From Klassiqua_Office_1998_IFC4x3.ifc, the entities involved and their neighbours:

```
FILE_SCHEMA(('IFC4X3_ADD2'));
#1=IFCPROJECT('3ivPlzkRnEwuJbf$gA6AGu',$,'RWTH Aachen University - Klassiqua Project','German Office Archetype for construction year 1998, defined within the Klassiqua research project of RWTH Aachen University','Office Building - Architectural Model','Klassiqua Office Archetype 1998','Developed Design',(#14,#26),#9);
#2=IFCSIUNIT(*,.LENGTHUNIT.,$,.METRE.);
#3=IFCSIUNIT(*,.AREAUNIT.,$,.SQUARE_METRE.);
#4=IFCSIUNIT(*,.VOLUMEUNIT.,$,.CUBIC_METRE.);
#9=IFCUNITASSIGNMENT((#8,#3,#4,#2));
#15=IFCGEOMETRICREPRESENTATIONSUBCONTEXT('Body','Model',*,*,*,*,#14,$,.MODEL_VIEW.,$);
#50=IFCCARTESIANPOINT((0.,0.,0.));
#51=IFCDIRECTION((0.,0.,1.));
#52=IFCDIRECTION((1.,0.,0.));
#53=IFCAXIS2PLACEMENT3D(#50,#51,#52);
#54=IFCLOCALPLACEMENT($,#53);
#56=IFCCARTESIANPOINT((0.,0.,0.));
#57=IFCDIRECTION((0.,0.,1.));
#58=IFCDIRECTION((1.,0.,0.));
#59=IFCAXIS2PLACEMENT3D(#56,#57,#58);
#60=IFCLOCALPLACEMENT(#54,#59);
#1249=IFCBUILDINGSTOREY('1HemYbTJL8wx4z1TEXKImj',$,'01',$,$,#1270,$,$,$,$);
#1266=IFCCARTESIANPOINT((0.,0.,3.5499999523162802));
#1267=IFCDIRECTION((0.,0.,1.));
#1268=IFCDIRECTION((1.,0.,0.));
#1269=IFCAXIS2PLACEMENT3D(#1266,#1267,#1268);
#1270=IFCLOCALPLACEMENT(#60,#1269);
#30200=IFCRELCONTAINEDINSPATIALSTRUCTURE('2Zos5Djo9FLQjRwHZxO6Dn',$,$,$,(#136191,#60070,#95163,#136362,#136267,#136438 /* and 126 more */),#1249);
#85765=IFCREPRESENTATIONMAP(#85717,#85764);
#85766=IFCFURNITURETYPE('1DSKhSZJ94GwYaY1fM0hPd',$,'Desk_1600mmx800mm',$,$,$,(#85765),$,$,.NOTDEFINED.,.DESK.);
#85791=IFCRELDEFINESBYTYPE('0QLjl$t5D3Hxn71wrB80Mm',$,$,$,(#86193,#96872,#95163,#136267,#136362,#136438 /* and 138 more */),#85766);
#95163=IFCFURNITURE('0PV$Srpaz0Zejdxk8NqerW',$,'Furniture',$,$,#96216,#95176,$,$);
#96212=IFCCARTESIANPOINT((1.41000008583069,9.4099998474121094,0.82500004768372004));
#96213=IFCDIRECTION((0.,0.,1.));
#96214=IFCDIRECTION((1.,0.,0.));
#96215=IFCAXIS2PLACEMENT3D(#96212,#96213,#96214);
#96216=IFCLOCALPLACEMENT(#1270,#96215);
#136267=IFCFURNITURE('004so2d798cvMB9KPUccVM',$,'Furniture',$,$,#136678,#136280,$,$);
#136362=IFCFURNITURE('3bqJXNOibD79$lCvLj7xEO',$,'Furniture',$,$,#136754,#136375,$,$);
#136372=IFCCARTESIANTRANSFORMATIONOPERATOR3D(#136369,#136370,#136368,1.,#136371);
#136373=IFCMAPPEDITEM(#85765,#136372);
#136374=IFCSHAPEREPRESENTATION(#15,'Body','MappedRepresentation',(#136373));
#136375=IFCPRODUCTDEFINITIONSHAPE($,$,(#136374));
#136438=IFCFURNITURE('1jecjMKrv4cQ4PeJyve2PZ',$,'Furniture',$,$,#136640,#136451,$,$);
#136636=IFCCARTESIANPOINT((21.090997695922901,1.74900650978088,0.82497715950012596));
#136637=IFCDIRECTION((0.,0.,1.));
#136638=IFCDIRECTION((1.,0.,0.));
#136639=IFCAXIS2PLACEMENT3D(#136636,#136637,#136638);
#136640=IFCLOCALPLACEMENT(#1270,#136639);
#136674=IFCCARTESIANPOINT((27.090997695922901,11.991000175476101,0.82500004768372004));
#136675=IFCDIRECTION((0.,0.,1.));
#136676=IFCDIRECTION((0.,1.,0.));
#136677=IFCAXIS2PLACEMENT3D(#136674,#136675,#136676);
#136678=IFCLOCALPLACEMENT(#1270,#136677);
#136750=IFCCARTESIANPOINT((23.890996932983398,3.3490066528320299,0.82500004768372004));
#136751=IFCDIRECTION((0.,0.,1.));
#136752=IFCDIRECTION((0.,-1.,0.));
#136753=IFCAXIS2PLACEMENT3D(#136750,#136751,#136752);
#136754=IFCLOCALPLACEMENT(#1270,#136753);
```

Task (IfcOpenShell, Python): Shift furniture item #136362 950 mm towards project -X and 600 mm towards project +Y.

```python
import ifcopenshell
import ifcopenshell.api.geometry
import ifcopenshell.util.placement

model = ifcopenshell.open("Klassiqua_Office_1998_IFC4x3.ifc")

item = model.by_guid("3bqJXNOibD79$lCvLj7xEO")
matrix = ifcopenshell.util.placement.get_local_placement(item.ObjectPlacement)
matrix[0, 3] -= 0.95
matrix[1, 3] += 0.6
ifcopenshell.api.geometry.edit_object_placement(model, product=item, matrix=matrix, is_si=False)

print(ifcopenshell.util.placement.get_local_placement(item.ObjectPlacement).round(3) + 0.0)

model.write("Klassiqua_Office_1998_IFC4x3_v2.ifc")
```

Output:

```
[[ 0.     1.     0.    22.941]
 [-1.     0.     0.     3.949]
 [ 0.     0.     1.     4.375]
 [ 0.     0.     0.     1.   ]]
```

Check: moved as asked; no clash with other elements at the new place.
